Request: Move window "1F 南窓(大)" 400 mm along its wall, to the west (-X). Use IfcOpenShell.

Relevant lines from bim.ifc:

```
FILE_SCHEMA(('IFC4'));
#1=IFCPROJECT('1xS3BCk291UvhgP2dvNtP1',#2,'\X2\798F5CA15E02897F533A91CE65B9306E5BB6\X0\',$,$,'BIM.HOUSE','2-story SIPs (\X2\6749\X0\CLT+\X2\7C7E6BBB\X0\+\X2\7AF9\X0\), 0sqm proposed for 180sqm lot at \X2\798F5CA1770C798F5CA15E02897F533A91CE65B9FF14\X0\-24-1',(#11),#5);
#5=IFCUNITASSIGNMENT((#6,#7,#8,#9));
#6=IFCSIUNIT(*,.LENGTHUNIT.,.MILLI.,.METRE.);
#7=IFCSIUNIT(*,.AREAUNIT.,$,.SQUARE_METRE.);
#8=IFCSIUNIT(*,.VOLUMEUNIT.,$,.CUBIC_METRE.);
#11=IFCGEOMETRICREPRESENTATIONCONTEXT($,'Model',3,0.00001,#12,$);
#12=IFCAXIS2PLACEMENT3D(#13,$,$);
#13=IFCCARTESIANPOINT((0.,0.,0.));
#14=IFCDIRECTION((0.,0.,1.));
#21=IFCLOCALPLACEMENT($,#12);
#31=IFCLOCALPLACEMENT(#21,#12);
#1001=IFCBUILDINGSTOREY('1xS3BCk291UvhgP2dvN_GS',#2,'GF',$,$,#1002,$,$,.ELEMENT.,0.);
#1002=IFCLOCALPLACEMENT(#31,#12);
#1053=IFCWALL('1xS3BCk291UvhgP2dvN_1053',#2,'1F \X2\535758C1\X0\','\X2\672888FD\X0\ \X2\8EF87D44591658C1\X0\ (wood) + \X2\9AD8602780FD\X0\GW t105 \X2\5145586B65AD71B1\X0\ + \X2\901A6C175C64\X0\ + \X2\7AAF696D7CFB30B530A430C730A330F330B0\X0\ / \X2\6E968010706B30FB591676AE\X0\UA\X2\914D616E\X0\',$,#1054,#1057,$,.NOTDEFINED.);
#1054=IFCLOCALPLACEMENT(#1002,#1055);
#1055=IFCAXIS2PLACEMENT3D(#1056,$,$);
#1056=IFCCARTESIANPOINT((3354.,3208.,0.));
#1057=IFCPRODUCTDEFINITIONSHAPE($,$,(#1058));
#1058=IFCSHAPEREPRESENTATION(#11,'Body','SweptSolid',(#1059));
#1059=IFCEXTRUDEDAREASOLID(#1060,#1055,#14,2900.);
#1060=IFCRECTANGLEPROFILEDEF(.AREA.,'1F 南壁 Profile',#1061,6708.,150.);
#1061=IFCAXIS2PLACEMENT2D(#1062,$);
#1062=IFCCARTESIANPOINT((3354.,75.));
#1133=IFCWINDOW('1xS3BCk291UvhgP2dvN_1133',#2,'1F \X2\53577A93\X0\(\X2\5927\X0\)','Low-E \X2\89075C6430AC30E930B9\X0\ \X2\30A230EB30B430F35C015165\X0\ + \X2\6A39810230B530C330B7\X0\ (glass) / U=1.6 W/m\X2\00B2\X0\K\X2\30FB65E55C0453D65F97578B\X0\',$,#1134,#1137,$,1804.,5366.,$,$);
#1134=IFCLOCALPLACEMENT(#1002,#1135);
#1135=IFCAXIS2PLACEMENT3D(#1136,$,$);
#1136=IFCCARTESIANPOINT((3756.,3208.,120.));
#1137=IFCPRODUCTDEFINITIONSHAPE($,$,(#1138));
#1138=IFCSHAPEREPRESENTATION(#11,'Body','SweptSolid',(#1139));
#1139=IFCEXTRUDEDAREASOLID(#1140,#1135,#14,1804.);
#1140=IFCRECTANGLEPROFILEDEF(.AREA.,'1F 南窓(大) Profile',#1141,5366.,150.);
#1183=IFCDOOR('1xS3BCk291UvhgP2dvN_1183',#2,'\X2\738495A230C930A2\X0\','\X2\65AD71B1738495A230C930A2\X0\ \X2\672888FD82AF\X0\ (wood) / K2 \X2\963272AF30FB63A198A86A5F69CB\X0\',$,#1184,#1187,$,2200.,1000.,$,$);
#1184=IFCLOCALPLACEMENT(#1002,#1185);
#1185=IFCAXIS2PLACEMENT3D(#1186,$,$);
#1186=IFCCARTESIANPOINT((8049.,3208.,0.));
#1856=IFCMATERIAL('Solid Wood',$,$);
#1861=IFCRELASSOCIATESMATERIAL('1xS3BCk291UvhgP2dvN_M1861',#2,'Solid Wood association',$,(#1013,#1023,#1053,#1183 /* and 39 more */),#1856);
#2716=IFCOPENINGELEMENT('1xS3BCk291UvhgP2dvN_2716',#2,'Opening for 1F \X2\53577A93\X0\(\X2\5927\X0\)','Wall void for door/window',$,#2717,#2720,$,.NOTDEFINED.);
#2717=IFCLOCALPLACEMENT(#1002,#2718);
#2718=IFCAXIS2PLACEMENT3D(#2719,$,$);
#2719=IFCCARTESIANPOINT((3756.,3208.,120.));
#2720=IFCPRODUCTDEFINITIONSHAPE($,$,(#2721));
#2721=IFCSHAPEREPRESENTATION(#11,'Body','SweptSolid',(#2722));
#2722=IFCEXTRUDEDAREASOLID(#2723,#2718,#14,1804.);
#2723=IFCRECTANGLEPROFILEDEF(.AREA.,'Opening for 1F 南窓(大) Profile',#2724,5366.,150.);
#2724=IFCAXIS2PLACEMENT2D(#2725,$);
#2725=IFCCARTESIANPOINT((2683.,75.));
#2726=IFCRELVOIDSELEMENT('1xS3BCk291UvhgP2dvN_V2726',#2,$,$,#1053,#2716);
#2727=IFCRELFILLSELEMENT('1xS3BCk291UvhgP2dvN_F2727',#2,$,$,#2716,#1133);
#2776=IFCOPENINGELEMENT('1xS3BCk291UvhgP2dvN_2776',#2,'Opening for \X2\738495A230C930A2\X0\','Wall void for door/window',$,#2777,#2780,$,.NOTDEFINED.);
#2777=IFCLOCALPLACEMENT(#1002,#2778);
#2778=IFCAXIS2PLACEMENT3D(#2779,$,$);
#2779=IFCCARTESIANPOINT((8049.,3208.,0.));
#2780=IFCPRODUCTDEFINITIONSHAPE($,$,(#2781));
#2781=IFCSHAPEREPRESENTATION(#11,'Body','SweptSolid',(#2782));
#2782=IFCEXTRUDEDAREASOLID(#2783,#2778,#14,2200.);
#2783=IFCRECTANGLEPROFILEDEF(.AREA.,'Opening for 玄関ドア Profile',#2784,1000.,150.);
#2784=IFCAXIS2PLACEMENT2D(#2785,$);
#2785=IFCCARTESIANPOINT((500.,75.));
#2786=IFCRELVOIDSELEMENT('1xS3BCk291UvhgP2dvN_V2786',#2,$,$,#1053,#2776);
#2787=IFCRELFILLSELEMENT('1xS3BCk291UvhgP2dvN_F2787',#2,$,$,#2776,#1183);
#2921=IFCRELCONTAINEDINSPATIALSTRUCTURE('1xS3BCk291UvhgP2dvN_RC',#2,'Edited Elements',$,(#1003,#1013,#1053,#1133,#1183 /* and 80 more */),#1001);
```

```python
import ifcopenshell
import ifcopenshell.api.geometry
import ifcopenshell.util.placement

model = ifcopenshell.open("bim.ifc")

window = model.by_id(1133)
opening = window.FillsVoids[0].RelatingOpeningElement
wall = opening.VoidsElements[0].RelatingBuildingElement

wall_matrix = ifcopenshell.util.placement.get_local_placement(wall.ObjectPlacement)
shift = wall_matrix[:3, 0] * -400.0
before = ifcopenshell.util.placement.get_local_placement(window.ObjectPlacement)[:3, 3].copy()

# The window is not placed relative to its opening, so move both.
for product in (opening, window):
    matrix = ifcopenshell.util.placement.get_local_placement(product.ObjectPlacement)
    matrix[:3, 3] += shift
    ifcopenshell.api.geometry.edit_object_placement(model, product=product, matrix=matrix, is_si=False)

after = ifcopenshell.util.placement.get_local_placement(window.ObjectPlacement)[:3, 3]
print("window moved by", (after - before).round(3) + 0.0)

model.write("bim_updated.ifc")
```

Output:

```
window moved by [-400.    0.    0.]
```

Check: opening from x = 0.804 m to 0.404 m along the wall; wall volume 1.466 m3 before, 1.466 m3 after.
